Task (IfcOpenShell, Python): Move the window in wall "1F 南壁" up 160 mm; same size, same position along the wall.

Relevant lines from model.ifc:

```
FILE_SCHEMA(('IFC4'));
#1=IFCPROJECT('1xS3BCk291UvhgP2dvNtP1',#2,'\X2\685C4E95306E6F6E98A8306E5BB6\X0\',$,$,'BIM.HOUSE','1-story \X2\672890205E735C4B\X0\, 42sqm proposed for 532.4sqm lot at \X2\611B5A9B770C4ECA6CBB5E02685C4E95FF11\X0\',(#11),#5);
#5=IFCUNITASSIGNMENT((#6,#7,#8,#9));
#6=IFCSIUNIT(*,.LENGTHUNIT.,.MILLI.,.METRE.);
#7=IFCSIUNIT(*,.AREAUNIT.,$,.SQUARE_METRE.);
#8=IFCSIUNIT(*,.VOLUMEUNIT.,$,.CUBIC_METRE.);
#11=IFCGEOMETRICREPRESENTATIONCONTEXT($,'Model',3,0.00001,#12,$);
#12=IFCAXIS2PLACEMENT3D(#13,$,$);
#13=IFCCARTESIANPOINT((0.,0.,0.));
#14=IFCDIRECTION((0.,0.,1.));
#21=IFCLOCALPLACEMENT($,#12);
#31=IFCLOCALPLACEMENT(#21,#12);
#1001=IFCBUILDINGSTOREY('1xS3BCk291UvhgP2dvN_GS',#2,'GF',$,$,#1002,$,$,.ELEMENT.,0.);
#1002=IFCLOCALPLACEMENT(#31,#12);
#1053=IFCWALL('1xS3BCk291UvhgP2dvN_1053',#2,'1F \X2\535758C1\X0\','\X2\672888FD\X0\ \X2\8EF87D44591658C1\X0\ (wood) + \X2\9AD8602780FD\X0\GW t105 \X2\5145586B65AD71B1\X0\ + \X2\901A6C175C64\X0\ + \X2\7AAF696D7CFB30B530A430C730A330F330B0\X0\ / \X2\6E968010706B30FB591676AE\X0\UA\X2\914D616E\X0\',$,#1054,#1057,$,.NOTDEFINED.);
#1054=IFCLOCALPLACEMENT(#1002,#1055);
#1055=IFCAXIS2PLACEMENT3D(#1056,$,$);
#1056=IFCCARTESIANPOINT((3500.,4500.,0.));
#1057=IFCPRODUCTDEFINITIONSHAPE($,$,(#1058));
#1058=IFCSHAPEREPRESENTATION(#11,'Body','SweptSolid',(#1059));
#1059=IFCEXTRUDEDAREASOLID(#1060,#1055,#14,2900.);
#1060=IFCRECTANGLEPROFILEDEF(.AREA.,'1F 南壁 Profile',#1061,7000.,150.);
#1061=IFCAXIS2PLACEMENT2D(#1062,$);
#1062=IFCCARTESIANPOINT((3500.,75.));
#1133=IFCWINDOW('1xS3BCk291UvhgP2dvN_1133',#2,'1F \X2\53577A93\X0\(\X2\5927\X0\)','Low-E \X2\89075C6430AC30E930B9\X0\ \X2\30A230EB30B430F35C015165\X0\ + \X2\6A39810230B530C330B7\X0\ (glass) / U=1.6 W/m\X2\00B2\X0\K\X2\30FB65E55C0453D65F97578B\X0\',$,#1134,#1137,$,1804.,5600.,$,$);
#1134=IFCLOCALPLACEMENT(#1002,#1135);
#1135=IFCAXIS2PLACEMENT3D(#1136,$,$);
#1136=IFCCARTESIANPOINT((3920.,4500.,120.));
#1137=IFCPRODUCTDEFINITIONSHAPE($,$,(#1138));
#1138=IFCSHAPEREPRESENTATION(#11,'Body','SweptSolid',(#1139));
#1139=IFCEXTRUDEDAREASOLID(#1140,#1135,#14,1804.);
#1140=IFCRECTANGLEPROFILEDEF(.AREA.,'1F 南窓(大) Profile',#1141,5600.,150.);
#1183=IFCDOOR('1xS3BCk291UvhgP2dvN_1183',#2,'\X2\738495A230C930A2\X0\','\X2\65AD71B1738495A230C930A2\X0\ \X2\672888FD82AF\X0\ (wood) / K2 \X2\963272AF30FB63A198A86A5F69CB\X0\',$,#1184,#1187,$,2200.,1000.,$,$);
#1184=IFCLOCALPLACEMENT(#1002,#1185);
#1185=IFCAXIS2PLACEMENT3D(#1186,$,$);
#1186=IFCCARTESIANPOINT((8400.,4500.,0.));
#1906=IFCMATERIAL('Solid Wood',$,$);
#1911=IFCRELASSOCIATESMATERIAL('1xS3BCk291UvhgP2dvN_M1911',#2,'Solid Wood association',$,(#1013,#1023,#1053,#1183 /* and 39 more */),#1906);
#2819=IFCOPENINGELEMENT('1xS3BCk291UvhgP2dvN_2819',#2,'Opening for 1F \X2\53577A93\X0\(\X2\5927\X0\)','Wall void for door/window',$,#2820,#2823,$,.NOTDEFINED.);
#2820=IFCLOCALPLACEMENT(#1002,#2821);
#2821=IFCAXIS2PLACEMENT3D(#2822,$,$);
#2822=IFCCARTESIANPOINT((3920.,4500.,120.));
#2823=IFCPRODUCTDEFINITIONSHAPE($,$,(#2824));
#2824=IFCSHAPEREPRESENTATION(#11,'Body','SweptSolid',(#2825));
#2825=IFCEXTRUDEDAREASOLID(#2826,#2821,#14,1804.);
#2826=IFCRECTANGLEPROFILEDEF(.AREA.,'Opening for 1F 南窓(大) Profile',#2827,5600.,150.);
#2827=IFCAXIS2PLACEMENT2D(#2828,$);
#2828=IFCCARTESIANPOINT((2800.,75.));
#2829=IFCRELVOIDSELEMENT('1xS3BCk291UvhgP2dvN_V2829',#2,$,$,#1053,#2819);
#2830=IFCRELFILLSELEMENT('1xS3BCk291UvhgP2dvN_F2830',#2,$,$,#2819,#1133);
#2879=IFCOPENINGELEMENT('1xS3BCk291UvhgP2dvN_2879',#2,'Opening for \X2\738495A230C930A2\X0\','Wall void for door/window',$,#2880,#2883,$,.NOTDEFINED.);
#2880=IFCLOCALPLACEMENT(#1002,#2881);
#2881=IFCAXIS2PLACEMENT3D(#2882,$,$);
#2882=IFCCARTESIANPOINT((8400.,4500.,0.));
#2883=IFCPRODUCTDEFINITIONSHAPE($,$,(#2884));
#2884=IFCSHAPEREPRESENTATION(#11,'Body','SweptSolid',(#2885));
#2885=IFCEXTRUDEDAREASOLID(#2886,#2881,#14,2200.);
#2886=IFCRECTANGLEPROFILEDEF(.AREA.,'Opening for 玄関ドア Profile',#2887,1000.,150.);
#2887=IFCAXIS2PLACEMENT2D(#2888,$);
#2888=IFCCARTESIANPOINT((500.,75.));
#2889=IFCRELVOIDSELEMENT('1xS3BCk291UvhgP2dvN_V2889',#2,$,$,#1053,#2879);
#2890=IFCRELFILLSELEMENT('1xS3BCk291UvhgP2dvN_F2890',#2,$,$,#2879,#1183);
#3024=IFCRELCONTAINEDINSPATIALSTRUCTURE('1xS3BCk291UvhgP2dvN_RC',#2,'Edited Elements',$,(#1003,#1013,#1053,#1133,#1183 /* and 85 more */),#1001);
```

```python
import numpy as np
import ifcopenshell
import ifcopenshell.api.geometry
import ifcopenshell.util.placement
import ifcopenshell.util.unit

model = ifcopenshell.open("model.ifc")
unit_scale = ifcopenshell.util.unit.calculate_unit_scale(model)

window = model.by_guid("1xS3BCk291UvhgP2dvN_1133")
opening = window.FillsVoids[0].RelatingOpeningElement
dz = 0.16 / unit_scale

shift = np.array([0.0, 0.0, dz])
# The window is not placed relative to its opening, so move both.
for product in (opening, window):
    matrix = ifcopenshell.util.placement.get_local_placement(product.ObjectPlacement)
    matrix[:3, 3] += shift
    ifcopenshell.api.geometry.edit_object_placement(model, product=product, matrix=matrix, is_si=False)

print(f"moved by {dz * unit_scale:+.3f} m")

model.write("model_updated.ifc")
```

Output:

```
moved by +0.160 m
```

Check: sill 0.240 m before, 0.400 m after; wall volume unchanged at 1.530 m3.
